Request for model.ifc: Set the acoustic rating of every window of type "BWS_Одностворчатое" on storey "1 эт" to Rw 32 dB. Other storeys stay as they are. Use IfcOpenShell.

First a look at what the model holds.

```python
import ifcopenshell
import ifcopenshell.util.element

model = ifcopenshell.open("model.ifc")
print(model.schema)
storey = next(s for s in model.by_type("IfcBuildingStorey") if s.Name == "1 эт")
windows = [e for e in ifcopenshell.util.element.get_decomposition(storey) if e.is_a("IfcWindow")]
seen = {}
for e in windows:
    element_type = ifcopenshell.util.element.get_type(e)
    key = (element_type.Name if element_type != e and element_type else None, ifcopenshell.util.element.get_pset(e, "Pset_WindowCommon", "AcousticRating"))
    seen[key] = seen.get(key, 0) + 1
for (name, value), count in sorted(seen.items(), key=str):
    print(count, "x", name, "|", value)
```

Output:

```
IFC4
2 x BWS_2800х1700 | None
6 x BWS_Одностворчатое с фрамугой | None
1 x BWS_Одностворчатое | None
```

```python
import ifcopenshell
import ifcopenshell.api.pset
import ifcopenshell.util.element

model = ifcopenshell.open("model.ifc")

storey = next(s for s in model.by_type("IfcBuildingStorey") if s.Name == "1 эт")
windows = [e for e in ifcopenshell.util.element.get_decomposition(storey) if e.is_a("IfcWindow")]

count = 0
for e in windows:
    element_type = ifcopenshell.util.element.get_type(e)
    if element_type in (None, e) or element_type.Name != "BWS_Одностворчатое":
        continue
    # add_pset returns the element's existing set when there is one.
    pset = ifcopenshell.api.pset.add_pset(model, product=e, name="Pset_WindowCommon")
    ifcopenshell.api.pset.edit_pset(model, pset=pset, properties={"AcousticRating": "Rw 32 dB"})
    count += 1

print(count, "windows updated")

model.write("model_updated.ifc")
```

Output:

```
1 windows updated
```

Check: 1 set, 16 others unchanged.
